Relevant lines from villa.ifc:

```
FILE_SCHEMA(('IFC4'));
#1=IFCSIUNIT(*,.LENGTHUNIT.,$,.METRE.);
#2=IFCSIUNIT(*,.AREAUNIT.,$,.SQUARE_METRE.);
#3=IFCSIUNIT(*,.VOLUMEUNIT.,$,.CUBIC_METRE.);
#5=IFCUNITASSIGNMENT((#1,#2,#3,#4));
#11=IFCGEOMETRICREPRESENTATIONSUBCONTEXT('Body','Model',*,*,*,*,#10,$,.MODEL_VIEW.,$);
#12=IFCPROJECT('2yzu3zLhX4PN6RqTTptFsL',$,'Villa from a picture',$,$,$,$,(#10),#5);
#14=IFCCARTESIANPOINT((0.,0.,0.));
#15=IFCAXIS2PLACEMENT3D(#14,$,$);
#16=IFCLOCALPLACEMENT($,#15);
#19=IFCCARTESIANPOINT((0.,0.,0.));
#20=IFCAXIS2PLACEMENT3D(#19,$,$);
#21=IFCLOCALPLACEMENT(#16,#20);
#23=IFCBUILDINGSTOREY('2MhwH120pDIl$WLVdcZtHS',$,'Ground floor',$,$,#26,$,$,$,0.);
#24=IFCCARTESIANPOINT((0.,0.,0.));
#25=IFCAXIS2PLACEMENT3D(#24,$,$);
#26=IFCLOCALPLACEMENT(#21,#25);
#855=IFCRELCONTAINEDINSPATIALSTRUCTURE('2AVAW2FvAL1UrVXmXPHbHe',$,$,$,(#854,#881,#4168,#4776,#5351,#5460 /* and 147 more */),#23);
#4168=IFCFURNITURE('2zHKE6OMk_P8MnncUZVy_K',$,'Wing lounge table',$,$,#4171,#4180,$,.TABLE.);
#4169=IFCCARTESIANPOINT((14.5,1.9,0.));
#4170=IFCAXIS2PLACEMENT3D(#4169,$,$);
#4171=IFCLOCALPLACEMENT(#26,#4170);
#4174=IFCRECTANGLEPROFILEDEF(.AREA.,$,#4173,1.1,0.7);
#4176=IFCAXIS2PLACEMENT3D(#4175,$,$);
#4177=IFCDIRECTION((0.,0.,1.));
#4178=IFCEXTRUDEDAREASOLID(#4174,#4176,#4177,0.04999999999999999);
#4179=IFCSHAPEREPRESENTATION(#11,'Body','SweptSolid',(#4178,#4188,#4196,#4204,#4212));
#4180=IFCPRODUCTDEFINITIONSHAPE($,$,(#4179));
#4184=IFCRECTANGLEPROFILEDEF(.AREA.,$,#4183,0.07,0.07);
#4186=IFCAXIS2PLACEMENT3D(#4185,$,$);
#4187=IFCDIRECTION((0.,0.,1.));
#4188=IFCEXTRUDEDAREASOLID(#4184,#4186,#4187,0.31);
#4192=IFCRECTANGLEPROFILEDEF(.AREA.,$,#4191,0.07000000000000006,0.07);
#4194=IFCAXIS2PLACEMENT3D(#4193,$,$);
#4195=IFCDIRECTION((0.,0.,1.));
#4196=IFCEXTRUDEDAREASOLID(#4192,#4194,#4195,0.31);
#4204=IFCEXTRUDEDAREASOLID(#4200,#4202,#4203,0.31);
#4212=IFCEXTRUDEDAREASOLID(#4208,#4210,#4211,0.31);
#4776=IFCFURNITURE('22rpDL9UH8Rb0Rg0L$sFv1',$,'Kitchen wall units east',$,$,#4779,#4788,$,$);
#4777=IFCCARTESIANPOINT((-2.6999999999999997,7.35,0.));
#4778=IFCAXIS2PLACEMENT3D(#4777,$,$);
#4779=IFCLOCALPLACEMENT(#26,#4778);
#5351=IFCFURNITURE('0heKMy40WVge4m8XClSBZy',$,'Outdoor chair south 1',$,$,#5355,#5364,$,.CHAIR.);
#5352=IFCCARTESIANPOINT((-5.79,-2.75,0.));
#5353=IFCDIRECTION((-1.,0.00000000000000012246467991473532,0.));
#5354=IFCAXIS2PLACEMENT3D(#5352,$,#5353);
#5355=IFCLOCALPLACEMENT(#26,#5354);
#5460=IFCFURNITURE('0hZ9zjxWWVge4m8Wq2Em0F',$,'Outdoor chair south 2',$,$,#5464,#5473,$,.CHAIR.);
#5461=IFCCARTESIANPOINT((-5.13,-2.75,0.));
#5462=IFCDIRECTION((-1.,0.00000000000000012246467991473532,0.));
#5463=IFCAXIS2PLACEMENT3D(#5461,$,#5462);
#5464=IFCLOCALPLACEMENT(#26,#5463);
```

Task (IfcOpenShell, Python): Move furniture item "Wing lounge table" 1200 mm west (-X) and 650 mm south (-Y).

```python
import ifcopenshell
import ifcopenshell.api.geometry
import ifcopenshell.util.placement

model = ifcopenshell.open("villa.ifc")

item = model.by_guid("2zHKE6OMk_P8MnncUZVy_K")
matrix = ifcopenshell.util.placement.get_local_placement(item.ObjectPlacement)
matrix[0, 3] -= 1.2
matrix[1, 3] -= 0.65
ifcopenshell.api.geometry.edit_object_placement(model, product=item, matrix=matrix, is_si=False)

print(ifcopenshell.util.placement.get_local_placement(item.ObjectPlacement).round(3) + 0.0)

model.write("villa-out.ifc")
```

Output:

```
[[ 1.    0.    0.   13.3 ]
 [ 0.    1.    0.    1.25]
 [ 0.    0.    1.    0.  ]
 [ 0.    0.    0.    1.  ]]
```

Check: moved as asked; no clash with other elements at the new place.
